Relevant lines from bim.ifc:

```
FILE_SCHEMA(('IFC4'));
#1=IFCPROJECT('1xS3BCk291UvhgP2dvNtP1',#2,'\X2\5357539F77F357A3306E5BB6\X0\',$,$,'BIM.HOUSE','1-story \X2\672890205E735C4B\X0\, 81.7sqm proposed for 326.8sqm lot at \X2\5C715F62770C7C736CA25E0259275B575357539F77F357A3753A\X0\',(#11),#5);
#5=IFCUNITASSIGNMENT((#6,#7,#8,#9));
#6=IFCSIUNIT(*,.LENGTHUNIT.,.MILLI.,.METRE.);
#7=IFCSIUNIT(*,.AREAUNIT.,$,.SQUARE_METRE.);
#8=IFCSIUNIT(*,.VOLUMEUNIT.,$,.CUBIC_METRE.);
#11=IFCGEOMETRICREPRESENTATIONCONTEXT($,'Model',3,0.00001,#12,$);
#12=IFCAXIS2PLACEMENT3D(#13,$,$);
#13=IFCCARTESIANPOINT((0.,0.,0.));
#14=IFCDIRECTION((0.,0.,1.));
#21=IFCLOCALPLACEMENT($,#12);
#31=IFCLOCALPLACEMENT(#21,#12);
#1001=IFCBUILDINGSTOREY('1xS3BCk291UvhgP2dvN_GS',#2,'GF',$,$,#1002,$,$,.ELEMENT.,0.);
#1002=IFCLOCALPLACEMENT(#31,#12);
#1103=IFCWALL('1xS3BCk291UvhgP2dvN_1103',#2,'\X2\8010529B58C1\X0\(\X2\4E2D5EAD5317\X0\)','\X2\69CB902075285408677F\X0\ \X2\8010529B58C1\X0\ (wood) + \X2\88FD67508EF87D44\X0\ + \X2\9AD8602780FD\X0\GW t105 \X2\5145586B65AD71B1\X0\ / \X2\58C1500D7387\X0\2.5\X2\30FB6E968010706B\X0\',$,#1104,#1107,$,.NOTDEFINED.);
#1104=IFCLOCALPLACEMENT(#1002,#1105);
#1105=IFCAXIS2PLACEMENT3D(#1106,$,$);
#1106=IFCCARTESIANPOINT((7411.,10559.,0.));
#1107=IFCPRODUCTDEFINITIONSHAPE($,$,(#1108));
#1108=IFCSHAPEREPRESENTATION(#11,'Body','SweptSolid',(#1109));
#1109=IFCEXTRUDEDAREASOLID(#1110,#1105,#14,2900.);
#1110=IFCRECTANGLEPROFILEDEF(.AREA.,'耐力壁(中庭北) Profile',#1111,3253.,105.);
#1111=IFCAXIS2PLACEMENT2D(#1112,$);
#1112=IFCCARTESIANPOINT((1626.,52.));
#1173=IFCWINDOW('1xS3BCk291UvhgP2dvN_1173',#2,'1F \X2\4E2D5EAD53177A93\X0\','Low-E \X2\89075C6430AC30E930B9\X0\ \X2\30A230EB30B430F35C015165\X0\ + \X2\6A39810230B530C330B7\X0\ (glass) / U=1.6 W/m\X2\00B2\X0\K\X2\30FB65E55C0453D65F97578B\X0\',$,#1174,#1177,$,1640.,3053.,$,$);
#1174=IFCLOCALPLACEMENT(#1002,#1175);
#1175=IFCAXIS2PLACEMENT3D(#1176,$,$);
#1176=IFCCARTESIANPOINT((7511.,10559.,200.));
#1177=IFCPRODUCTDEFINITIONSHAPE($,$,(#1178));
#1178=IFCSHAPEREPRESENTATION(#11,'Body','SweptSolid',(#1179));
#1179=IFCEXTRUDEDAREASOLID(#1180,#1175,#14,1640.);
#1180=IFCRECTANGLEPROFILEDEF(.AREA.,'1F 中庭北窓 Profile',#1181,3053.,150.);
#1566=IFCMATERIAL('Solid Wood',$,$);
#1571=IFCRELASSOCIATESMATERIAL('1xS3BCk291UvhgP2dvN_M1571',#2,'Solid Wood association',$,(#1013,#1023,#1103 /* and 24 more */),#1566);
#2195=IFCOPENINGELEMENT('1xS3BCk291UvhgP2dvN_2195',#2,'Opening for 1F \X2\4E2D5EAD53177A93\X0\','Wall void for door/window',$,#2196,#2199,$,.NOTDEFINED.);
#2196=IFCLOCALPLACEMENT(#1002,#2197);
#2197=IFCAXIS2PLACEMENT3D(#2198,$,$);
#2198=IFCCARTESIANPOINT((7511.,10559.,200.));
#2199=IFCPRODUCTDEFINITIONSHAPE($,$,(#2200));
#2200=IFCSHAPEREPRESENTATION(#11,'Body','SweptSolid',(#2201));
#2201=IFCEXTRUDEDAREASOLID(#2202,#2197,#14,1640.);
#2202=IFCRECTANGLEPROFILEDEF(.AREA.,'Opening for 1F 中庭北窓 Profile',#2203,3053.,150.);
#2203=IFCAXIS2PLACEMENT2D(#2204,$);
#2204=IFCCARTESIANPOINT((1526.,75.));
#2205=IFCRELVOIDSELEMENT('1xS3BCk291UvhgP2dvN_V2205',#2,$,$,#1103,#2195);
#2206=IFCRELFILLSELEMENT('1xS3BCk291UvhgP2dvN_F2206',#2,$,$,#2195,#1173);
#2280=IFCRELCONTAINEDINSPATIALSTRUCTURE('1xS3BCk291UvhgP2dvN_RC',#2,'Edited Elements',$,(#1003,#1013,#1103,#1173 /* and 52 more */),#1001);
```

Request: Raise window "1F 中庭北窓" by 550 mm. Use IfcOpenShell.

```python
import numpy as np
import ifcopenshell
import ifcopenshell.api.geometry
import ifcopenshell.util.placement
import ifcopenshell.util.unit

model = ifcopenshell.open("bim.ifc")
unit_scale = ifcopenshell.util.unit.calculate_unit_scale(model)

window = model.by_guid("1xS3BCk291UvhgP2dvN_1173")
opening = window.FillsVoids[0].RelatingOpeningElement
dz = 0.55 / unit_scale

shift = np.array([0.0, 0.0, dz])
# The window is not placed relative to its opening, so move both.
for product in (opening, window):
    matrix = ifcopenshell.util.placement.get_local_placement(product.ObjectPlacement)
    matrix[:3, 3] += shift
    ifcopenshell.api.geometry.edit_object_placement(model, product=product, matrix=matrix, is_si=False)

print(f"moved by {dz * unit_scale:+.3f} m")

model.write("bim-out.ifc")
```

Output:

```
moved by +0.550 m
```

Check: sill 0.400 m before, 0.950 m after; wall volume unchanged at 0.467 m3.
